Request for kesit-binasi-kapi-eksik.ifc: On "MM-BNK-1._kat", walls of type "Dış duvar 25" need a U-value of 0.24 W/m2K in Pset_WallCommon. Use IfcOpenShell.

First a look at what the model holds.

```python
import ifcopenshell
import ifcopenshell.util.element

model = ifcopenshell.open("kesit-binasi-kapi-eksik.ifc")
print(model.schema)
storey = next(s for s in model.by_type("IfcBuildingStorey") if s.Name == "MM-BNK-1._kat")
walls = [e for e in ifcopenshell.util.element.get_decomposition(storey) if e.is_a("IfcWall")]
seen = {}
for e in walls:
    element_type = ifcopenshell.util.element.get_type(e)
    key = (element_type.Name if element_type != e and element_type else None, ifcopenshell.util.element.get_pset(e, "Pset_WallCommon", "ThermalTransmittance"))
    seen[key] = seen.get(key, 0) + 1
for (name, value), count in sorted(seen.items(), key=str):
    print(count, "x", name, "|", value)
```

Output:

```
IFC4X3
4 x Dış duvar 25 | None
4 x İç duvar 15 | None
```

```python
import ifcopenshell
import ifcopenshell.api.pset
import ifcopenshell.util.element

model = ifcopenshell.open("kesit-binasi-kapi-eksik.ifc")

storey = next(s for s in model.by_type("IfcBuildingStorey") if s.Name == "MM-BNK-1._kat")
walls = [e for e in ifcopenshell.util.element.get_decomposition(storey) if e.is_a("IfcWall")]

count = 0
for e in walls:
    element_type = ifcopenshell.util.element.get_type(e)
    if element_type in (None, e) or element_type.Name != "Dış duvar 25":
        continue
    # add_pset returns the element's existing set when there is one.
    pset = ifcopenshell.api.pset.add_pset(model, product=e, name="Pset_WallCommon")
    ifcopenshell.api.pset.edit_pset(model, pset=pset, properties={"ThermalTransmittance": 0.24})
    count += 1

print(count, "walls updated")

model.write("kesit-binasi-kapi-eksik_updated.ifc")
```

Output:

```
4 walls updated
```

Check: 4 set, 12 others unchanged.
